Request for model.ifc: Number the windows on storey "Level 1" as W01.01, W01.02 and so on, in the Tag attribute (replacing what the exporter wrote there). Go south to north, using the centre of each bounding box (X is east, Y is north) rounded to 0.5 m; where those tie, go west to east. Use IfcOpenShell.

First a look at what the model holds.

```python
import ifcopenshell
import ifcopenshell.util.element
import ifcopenshell.util.placement

model = ifcopenshell.open("model.ifc")
print(model.schema)
storey = next(s for s in model.by_type("IfcBuildingStorey") if s.Name == "Level 1")
windows = [e for e in ifcopenshell.util.element.get_decomposition(storey) if e.is_a("IfcWindow")]
for e in sorted(windows, key=lambda e: e.id()):
    origin = ifcopenshell.util.placement.get_local_placement(e.ObjectPlacement)[:3, 3]
    print(e.id(), e.Tag, e.Name, origin.round(2) + 0.0, sep=" | ")
```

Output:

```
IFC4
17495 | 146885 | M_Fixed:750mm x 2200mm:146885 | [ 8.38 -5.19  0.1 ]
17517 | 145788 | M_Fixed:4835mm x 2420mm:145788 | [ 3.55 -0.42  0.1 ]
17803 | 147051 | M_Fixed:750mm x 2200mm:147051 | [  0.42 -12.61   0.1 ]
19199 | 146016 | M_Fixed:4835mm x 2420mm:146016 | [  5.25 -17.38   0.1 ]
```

```python
import ifcopenshell
import ifcopenshell.geom
import ifcopenshell.util.element
import ifcopenshell.util.shape

model = ifcopenshell.open("model.ifc")
settings = ifcopenshell.geom.settings()
settings.set("use-world-coords", True)


def centre(element):
    shape = ifcopenshell.geom.create_shape(settings, element)
    return ifcopenshell.util.shape.get_bbox_centroid(shape.geometry)


storey = next(s for s in model.by_type("IfcBuildingStorey") if s.Name == "Level 1")
windows = [e for e in ifcopenshell.util.element.get_decomposition(storey) if e.is_a("IfcWindow")]

# Insertion points can sit at a corner or the storey origin, so sort by the geometry (in metres).
centres = {e: centre(e) for e in windows}
windows.sort(key=lambda e: (round(centres[e][1] / 0.5), centres[e][0]))

for i, e in enumerate(windows, start=1):
    number = f"W01.{i:02d}"
    e.Tag = number
    print(e.id(), number)

model.write("model_rev.ifc")
```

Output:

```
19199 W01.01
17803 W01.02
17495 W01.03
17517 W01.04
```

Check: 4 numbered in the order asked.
